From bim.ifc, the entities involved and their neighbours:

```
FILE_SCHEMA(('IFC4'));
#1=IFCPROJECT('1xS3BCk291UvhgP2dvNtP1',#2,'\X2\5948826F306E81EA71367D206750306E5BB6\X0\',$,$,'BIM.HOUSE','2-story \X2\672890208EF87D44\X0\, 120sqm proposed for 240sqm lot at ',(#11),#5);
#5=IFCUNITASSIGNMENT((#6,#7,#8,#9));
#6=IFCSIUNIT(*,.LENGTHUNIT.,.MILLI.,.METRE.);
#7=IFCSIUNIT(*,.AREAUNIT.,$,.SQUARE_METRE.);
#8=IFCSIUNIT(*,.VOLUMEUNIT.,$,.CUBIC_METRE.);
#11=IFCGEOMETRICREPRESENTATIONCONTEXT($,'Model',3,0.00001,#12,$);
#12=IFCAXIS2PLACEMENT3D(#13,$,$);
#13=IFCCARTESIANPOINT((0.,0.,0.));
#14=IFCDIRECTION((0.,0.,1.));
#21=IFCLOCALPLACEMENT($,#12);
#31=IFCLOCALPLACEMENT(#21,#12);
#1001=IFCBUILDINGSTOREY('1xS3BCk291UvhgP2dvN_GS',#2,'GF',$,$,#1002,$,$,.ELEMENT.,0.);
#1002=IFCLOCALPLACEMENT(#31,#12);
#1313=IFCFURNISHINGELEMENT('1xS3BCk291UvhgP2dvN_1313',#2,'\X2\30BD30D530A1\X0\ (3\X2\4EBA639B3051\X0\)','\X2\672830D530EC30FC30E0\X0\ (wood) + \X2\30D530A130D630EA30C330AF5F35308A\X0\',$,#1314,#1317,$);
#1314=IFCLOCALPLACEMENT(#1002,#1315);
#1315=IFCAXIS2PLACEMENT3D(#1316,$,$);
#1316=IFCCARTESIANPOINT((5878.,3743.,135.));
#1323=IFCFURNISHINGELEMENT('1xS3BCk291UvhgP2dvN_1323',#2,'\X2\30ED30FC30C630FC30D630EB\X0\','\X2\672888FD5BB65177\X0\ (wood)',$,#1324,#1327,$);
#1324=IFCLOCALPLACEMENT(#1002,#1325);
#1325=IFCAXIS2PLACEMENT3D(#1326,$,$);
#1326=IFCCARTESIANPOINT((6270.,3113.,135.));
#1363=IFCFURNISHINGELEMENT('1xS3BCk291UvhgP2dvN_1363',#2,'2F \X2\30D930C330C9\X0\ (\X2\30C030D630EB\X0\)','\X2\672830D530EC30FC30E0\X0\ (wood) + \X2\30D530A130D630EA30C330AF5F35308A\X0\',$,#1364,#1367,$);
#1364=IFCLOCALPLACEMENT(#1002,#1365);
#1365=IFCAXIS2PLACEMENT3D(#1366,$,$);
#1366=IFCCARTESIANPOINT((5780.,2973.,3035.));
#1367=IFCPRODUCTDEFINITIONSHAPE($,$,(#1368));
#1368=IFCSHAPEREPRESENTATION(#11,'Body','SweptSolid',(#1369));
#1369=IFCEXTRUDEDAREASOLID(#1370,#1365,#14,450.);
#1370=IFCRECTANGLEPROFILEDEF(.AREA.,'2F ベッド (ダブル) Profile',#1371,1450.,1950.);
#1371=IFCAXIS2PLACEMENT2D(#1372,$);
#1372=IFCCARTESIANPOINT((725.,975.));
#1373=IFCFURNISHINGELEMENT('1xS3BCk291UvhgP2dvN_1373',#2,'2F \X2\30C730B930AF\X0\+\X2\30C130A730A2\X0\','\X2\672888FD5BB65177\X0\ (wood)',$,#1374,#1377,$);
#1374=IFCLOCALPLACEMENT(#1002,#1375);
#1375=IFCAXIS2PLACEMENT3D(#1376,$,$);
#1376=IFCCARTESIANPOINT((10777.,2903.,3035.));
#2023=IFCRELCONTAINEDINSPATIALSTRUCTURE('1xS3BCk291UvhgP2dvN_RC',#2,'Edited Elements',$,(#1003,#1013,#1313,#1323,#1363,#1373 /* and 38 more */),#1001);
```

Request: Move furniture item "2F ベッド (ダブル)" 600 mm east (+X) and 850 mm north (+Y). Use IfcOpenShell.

```python
import ifcopenshell
import ifcopenshell.api.geometry
import ifcopenshell.util.placement

model = ifcopenshell.open("bim.ifc")

item = model.by_guid("1xS3BCk291UvhgP2dvN_1363")
matrix = ifcopenshell.util.placement.get_local_placement(item.ObjectPlacement)
matrix[0, 3] += 600.0
matrix[1, 3] += 850.0
ifcopenshell.api.geometry.edit_object_placement(model, product=item, matrix=matrix, is_si=False)

print(ifcopenshell.util.placement.get_local_placement(item.ObjectPlacement).round(3) + 0.0)

model.write("bim-out.ifc")
```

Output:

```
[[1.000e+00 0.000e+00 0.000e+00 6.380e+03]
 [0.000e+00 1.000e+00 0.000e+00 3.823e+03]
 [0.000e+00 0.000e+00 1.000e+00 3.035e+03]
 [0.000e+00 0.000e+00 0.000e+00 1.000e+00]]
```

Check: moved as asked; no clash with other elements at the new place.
